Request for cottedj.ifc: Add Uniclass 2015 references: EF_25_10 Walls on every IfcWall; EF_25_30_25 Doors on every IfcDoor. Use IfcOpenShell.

First a look at what the model holds.

```python
import ifcopenshell

model = ifcopenshell.open("cottedj.ifc")
print(model.schema)
print("classifications:", [c.Name for c in model.by_type("IfcClassification")])
for ifc_class in ("IfcDoor", "IfcRoof", "IfcStair", "IfcWall", "IfcWindow"):
    print(ifc_class, len(model.by_type(ifc_class)))
```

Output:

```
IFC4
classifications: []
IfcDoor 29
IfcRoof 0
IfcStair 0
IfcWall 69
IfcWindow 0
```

```python
import ifcopenshell
import ifcopenshell.api.classification

model = ifcopenshell.open("cottedj.ifc")

system = ifcopenshell.api.classification.add_classification(model, classification="Uniclass 2015")

codes = {
    "IfcWall": ("EF_25_10", "Walls"),
    "IfcDoor": ("EF_25_30_25", "Doors"),
}
for ifc_class, (code, name) in codes.items():
    products = model.by_type(ifc_class)
    ifcopenshell.api.classification.add_reference(
        model, products=products, classification=system, identification=code, name=name
    )
    print(code, len(products))

model.write("cottedj_edited.ifc")
```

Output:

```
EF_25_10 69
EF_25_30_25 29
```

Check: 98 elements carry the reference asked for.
